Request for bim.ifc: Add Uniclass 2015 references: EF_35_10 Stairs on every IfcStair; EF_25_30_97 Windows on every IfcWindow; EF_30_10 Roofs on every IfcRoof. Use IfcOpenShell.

First a look at what the model holds.

```python
import ifcopenshell

model = ifcopenshell.open("bim.ifc")
print(model.schema)
print("classifications:", [c.Name for c in model.by_type("IfcClassification")])
for ifc_class in ("IfcDoor", "IfcRoof", "IfcStair", "IfcWall", "IfcWindow"):
    print(ifc_class, len(model.by_type(ifc_class)))
```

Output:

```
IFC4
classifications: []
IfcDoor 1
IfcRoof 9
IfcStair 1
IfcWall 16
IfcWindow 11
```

```python
import ifcopenshell
import ifcopenshell.api.classification

model = ifcopenshell.open("bim.ifc")

system = ifcopenshell.api.classification.add_classification(model, classification="Uniclass 2015")

codes = {
    "IfcStair": ("EF_35_10", "Stairs"),
    "IfcWindow": ("EF_25_30_97", "Windows"),
    "IfcRoof": ("EF_30_10", "Roofs"),
}
for ifc_class, (code, name) in codes.items():
    products = model.by_type(ifc_class)
    ifcopenshell.api.classification.add_reference(
        model, products=products, classification=system, identification=code, name=name
    )
    print(code, len(products))

model.write("bim_edited.ifc")
```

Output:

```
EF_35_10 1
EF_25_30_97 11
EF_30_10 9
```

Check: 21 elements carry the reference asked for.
